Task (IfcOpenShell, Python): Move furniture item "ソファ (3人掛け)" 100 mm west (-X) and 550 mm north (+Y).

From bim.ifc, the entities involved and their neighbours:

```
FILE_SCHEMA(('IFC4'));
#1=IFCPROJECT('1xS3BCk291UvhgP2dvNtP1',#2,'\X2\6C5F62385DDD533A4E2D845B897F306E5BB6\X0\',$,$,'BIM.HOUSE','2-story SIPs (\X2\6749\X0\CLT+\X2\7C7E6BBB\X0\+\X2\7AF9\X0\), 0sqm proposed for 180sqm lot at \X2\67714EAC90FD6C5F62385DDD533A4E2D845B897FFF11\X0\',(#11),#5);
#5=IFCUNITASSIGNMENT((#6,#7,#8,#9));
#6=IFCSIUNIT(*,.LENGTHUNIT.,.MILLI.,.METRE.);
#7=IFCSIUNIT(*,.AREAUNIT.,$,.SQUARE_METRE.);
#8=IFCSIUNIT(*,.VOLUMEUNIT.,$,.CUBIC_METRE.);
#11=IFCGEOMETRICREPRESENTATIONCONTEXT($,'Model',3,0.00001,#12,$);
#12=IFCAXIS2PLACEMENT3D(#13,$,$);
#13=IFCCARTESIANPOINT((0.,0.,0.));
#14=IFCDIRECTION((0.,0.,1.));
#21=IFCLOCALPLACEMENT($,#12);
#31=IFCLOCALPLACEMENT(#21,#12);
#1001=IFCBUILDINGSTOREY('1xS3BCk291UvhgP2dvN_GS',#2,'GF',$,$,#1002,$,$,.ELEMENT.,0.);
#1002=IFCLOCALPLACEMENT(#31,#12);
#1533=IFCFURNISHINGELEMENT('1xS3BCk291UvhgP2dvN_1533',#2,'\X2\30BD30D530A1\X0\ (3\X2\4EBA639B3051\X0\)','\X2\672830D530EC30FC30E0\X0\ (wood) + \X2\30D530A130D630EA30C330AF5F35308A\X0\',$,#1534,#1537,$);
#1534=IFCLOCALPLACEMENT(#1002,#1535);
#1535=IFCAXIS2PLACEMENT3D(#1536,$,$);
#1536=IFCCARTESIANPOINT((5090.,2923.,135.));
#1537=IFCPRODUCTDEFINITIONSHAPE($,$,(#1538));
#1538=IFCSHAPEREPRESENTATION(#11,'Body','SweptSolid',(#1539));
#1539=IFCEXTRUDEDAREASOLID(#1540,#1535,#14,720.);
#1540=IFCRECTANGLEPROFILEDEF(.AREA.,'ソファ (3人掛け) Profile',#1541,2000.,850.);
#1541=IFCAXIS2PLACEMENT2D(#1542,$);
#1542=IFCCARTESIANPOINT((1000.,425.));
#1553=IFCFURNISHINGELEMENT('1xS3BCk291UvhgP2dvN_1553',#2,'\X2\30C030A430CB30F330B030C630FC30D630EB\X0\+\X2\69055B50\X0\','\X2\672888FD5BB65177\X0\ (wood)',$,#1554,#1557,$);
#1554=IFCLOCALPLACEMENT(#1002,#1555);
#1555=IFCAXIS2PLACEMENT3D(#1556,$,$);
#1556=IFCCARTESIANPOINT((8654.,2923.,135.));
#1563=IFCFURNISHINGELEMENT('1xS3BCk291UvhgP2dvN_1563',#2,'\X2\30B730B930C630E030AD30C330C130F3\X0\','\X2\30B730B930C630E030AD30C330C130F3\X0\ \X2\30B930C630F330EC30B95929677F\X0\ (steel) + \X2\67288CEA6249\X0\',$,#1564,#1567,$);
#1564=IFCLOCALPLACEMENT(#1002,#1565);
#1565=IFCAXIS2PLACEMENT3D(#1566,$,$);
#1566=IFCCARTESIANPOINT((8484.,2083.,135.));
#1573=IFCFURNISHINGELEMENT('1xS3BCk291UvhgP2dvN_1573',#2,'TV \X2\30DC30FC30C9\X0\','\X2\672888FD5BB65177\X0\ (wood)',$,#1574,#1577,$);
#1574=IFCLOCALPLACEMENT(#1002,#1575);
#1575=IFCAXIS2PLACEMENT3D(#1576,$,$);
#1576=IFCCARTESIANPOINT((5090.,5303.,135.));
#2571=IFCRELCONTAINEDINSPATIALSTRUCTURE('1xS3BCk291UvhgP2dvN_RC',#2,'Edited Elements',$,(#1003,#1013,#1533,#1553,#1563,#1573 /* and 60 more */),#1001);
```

```python
import ifcopenshell
import ifcopenshell.api.geometry
import ifcopenshell.util.placement
import ifcopenshell.util.unit

model = ifcopenshell.open("bim.ifc")
unit_scale = ifcopenshell.util.unit.calculate_unit_scale(model)

item = model.by_id(1533)
matrix = ifcopenshell.util.placement.get_local_placement(item.ObjectPlacement)
matrix[0, 3] -= 0.1 / unit_scale
matrix[1, 3] += 0.55 / unit_scale
ifcopenshell.api.geometry.edit_object_placement(model, product=item, matrix=matrix, is_si=False)

print(ifcopenshell.util.placement.get_local_placement(item.ObjectPlacement).round(3) + 0.0)

model.write("bim_edited.ifc")
```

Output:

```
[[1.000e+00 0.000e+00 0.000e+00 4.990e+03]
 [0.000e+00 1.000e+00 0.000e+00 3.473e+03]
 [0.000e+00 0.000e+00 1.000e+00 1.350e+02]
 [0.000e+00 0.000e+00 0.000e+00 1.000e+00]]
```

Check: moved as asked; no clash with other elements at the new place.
